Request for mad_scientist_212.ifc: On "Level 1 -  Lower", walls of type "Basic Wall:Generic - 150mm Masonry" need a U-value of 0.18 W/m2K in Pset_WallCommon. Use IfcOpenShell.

First a look at what the model holds.

```python
import ifcopenshell
import ifcopenshell.util.element

model = ifcopenshell.open("mad_scientist_212.ifc")
print(model.schema)
storey = next(s for s in model.by_type("IfcBuildingStorey") if s.Name == "Level 1 -  Lower")
walls = [e for e in ifcopenshell.util.element.get_decomposition(storey) if e.is_a("IfcWall")]
seen = {}
for e in walls:
    element_type = ifcopenshell.util.element.get_type(e)
    key = (element_type.Name if element_type != e and element_type else None, ifcopenshell.util.element.get_pset(e, "Pset_WallCommon", "ThermalTransmittance"))
    seen[key] = seen.get(key, 0) + 1
for (name, value), count in sorted(seen.items(), key=str):
    print(count, "x", name, "|", value)
```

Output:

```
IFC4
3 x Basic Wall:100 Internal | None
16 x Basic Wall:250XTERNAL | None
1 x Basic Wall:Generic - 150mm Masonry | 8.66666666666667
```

```python
import ifcopenshell
import ifcopenshell.api.pset
import ifcopenshell.util.element

model = ifcopenshell.open("mad_scientist_212.ifc")

storey = next(s for s in model.by_type("IfcBuildingStorey") if s.Name == "Level 1 -  Lower")
walls = [e for e in ifcopenshell.util.element.get_decomposition(storey) if e.is_a("IfcWall")]

count = 0
for e in walls:
    element_type = ifcopenshell.util.element.get_type(e)
    if element_type in (None, e) or element_type.Name != "Basic Wall:Generic - 150mm Masonry":
        continue
    # add_pset returns the element's existing set when there is one.
    pset = ifcopenshell.api.pset.add_pset(model, product=e, name="Pset_WallCommon")
    ifcopenshell.api.pset.edit_pset(model, pset=pset, properties={"ThermalTransmittance": 0.18})
    count += 1

print(count, "walls updated")

model.write("mad_scientist_212_v2.ifc")
```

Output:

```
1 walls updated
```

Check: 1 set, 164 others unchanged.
